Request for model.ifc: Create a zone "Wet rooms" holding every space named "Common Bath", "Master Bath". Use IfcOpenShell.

First a look at what the model holds.

```python
import ifcopenshell

model = ifcopenshell.open("model.ifc")
print(model.schema)
seen = {}
for space in model.by_type("IfcSpace"):
    seen[space.LongName] = seen.get(space.LongName, 0) + 1
for name, count in sorted(seen.items(), key=str):
    print(count, "x", name)
print("zones:", [z.Name for z in model.by_type("IfcZone")][:20])
```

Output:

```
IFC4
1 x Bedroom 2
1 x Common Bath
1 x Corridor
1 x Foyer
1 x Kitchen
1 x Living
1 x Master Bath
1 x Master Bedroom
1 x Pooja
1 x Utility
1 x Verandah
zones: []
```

```python
import ifcopenshell
import ifcopenshell.api.group
import ifcopenshell.api.root

model = ifcopenshell.open("model.ifc")

names = {"Common Bath", "Master Bath"}
spaces = [s for s in model.by_type("IfcSpace") if s.LongName in names]

zone = ifcopenshell.api.root.create_entity(model, ifc_class="IfcZone", name="Wet rooms")
ifcopenshell.api.group.assign_group(model, products=spaces, group=zone)
print(len(spaces), "spaces in", zone.Name)

model.write("model_updated.ifc")
```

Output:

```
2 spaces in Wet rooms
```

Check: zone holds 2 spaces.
